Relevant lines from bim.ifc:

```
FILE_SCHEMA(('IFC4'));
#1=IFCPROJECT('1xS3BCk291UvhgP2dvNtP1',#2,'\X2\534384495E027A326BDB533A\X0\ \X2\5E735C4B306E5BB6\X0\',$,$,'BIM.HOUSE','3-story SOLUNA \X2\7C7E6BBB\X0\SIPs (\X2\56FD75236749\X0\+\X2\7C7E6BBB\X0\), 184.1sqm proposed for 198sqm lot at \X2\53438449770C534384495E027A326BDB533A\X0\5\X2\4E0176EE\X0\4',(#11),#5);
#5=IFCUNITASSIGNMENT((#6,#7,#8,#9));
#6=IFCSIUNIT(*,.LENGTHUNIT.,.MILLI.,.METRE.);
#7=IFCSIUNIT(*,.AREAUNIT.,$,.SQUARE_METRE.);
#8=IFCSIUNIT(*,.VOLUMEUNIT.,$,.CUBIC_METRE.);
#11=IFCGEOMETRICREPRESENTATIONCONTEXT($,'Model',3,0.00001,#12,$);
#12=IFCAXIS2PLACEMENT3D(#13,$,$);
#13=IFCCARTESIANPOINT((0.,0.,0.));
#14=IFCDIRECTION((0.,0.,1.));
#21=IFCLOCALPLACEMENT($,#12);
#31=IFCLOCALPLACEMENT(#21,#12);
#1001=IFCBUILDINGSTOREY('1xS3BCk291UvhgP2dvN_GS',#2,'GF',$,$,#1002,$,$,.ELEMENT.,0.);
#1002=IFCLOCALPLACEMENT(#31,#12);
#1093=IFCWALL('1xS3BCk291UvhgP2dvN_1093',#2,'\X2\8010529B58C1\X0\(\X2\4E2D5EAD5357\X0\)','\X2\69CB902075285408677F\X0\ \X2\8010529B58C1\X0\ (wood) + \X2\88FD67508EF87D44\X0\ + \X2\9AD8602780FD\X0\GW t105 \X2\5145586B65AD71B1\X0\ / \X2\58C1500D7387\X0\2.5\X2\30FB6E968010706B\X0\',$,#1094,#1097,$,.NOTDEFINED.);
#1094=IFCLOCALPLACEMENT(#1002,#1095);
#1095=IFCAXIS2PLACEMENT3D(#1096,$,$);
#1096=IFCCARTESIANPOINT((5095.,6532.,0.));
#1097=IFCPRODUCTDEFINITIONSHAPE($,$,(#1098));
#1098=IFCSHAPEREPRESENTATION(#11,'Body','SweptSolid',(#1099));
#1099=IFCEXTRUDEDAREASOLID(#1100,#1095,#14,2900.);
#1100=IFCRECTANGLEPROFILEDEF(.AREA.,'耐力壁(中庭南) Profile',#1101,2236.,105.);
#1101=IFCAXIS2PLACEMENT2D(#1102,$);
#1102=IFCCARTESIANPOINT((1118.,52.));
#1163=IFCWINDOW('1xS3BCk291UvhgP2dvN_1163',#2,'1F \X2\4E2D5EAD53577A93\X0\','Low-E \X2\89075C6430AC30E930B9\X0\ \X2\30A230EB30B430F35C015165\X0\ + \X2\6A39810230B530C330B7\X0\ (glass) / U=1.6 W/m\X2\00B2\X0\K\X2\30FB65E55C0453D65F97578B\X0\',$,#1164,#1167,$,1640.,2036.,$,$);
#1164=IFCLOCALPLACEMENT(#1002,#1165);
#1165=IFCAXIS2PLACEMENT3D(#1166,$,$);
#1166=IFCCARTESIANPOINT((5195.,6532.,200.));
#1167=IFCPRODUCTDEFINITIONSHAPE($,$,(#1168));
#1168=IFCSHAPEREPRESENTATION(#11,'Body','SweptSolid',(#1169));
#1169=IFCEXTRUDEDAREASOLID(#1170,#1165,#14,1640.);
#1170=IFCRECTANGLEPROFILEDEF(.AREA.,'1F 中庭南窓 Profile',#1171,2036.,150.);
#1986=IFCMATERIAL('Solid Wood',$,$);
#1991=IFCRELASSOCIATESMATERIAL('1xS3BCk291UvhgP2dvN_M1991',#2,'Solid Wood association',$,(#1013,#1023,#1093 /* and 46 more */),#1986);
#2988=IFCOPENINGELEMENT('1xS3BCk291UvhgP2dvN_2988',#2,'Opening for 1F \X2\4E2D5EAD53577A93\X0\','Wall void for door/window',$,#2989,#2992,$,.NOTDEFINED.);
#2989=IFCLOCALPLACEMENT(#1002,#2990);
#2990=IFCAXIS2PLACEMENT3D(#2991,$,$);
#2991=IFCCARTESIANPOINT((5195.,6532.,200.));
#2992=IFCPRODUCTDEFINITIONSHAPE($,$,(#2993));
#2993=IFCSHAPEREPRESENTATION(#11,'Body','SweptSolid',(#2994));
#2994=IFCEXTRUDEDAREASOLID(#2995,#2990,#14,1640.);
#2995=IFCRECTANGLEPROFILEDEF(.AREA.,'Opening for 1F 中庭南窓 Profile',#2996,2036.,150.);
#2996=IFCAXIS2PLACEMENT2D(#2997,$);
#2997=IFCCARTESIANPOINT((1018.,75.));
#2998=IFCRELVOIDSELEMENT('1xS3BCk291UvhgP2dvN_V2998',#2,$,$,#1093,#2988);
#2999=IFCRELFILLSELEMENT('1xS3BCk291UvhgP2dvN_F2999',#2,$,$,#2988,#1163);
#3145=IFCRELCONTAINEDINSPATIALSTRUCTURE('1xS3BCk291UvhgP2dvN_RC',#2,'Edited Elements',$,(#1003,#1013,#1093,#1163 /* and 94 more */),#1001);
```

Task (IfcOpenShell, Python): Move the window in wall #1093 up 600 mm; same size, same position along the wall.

```python
import numpy as np
import ifcopenshell
import ifcopenshell.api.geometry
import ifcopenshell.util.placement
import ifcopenshell.util.unit

model = ifcopenshell.open("bim.ifc")
unit_scale = ifcopenshell.util.unit.calculate_unit_scale(model)

window = model.by_guid("1xS3BCk291UvhgP2dvN_1163")
opening = window.FillsVoids[0].RelatingOpeningElement
dz = 600.0

shift = np.array([0.0, 0.0, dz])
# The window is not placed relative to its opening, so move both.
for product in (opening, window):
    matrix = ifcopenshell.util.placement.get_local_placement(product.ObjectPlacement)
    matrix[:3, 3] += shift
    ifcopenshell.api.geometry.edit_object_placement(model, product=product, matrix=matrix, is_si=False)

print(f"moved by {dz * unit_scale:+.3f} m")

model.write("bim_rev.ifc")
```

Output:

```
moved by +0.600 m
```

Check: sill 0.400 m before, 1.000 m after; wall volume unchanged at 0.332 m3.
